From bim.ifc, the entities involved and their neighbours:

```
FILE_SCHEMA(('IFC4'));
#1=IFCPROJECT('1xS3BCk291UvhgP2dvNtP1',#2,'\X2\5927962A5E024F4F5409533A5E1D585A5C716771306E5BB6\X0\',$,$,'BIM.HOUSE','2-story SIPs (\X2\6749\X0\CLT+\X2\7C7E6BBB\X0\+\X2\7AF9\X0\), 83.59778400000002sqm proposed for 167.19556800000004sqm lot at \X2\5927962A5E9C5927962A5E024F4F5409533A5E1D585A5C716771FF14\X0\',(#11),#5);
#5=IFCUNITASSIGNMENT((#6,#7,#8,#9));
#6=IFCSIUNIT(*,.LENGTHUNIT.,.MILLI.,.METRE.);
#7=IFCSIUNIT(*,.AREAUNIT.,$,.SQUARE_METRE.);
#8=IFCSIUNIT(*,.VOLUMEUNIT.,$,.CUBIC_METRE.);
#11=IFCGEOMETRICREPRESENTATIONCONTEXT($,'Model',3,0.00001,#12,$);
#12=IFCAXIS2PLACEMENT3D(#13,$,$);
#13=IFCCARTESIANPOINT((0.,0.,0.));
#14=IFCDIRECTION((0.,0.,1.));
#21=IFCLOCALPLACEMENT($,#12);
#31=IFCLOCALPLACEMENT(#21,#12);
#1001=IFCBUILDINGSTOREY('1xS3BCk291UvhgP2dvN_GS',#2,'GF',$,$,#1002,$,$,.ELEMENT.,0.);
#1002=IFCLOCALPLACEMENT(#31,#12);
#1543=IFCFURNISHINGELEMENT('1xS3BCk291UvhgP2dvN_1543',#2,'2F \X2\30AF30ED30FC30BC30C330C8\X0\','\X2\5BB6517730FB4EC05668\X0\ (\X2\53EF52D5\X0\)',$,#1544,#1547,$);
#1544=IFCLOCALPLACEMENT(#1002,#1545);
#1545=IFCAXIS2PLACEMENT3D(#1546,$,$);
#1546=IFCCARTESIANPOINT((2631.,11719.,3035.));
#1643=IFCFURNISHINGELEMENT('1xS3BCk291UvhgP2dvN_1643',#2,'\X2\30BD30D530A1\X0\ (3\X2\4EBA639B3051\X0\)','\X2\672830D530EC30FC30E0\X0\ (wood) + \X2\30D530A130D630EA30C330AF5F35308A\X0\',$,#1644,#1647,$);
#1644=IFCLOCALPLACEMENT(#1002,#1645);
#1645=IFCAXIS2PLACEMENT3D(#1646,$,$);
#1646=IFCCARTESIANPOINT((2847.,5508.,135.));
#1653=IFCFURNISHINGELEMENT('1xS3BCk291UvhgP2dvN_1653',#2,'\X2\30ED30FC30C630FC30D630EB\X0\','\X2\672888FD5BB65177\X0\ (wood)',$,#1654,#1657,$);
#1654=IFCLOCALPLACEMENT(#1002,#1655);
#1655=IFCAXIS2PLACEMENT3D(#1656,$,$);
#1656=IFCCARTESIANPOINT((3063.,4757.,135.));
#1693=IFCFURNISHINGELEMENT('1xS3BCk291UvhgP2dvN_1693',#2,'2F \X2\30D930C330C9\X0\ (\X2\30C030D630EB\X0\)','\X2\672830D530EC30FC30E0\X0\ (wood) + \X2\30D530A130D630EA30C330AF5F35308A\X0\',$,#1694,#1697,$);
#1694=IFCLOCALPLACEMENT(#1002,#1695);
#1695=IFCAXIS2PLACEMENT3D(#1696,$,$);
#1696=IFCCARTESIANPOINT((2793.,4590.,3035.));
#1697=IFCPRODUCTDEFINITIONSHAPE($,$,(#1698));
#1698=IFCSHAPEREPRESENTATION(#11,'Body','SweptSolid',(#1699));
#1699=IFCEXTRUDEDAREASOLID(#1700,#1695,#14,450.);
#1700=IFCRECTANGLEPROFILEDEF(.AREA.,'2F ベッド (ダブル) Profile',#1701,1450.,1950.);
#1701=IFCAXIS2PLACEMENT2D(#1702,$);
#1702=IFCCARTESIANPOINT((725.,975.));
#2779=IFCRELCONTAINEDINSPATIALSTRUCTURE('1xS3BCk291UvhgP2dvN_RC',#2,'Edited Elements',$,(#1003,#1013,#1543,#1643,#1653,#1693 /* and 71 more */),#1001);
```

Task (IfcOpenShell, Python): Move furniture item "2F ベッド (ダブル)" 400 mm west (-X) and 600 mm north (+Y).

```python
import ifcopenshell
import ifcopenshell.api.geometry
import ifcopenshell.util.placement
import ifcopenshell.util.unit

model = ifcopenshell.open("bim.ifc")
unit_scale = ifcopenshell.util.unit.calculate_unit_scale(model)

item = model.by_guid("1xS3BCk291UvhgP2dvN_1693")
matrix = ifcopenshell.util.placement.get_local_placement(item.ObjectPlacement)
matrix[0, 3] -= 0.4 / unit_scale
matrix[1, 3] += 0.6 / unit_scale
ifcopenshell.api.geometry.edit_object_placement(model, product=item, matrix=matrix, is_si=False)

print(ifcopenshell.util.placement.get_local_placement(item.ObjectPlacement).round(3) + 0.0)

model.write("bim_rev.ifc")
```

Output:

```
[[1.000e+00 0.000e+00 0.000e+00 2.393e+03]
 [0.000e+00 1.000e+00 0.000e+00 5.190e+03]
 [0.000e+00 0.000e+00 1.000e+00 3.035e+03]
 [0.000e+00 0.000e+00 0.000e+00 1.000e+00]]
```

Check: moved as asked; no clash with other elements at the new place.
